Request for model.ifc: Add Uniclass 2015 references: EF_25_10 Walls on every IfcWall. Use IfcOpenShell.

First a look at what the model holds.

```python
import ifcopenshell

model = ifcopenshell.open("model.ifc")
print(model.schema)
print("classifications:", [c.Name for c in model.by_type("IfcClassification")])
for ifc_class in ("IfcDoor", "IfcRoof", "IfcStair", "IfcWall", "IfcWindow"):
    print(ifc_class, len(model.by_type(ifc_class)))
```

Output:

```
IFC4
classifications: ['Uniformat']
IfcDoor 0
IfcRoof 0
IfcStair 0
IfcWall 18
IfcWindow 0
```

```python
import ifcopenshell
import ifcopenshell.api.classification

model = ifcopenshell.open("model.ifc")

system = ifcopenshell.api.classification.add_classification(model, classification="Uniclass 2015")

codes = {
    "IfcWall": ("EF_25_10", "Walls"),
}
for ifc_class, (code, name) in codes.items():
    products = model.by_type(ifc_class)
    ifcopenshell.api.classification.add_reference(
        model, products=products, classification=system, identification=code, name=name
    )
    print(code, len(products))

model.write("model_rev.ifc")
```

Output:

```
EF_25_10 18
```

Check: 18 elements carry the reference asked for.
